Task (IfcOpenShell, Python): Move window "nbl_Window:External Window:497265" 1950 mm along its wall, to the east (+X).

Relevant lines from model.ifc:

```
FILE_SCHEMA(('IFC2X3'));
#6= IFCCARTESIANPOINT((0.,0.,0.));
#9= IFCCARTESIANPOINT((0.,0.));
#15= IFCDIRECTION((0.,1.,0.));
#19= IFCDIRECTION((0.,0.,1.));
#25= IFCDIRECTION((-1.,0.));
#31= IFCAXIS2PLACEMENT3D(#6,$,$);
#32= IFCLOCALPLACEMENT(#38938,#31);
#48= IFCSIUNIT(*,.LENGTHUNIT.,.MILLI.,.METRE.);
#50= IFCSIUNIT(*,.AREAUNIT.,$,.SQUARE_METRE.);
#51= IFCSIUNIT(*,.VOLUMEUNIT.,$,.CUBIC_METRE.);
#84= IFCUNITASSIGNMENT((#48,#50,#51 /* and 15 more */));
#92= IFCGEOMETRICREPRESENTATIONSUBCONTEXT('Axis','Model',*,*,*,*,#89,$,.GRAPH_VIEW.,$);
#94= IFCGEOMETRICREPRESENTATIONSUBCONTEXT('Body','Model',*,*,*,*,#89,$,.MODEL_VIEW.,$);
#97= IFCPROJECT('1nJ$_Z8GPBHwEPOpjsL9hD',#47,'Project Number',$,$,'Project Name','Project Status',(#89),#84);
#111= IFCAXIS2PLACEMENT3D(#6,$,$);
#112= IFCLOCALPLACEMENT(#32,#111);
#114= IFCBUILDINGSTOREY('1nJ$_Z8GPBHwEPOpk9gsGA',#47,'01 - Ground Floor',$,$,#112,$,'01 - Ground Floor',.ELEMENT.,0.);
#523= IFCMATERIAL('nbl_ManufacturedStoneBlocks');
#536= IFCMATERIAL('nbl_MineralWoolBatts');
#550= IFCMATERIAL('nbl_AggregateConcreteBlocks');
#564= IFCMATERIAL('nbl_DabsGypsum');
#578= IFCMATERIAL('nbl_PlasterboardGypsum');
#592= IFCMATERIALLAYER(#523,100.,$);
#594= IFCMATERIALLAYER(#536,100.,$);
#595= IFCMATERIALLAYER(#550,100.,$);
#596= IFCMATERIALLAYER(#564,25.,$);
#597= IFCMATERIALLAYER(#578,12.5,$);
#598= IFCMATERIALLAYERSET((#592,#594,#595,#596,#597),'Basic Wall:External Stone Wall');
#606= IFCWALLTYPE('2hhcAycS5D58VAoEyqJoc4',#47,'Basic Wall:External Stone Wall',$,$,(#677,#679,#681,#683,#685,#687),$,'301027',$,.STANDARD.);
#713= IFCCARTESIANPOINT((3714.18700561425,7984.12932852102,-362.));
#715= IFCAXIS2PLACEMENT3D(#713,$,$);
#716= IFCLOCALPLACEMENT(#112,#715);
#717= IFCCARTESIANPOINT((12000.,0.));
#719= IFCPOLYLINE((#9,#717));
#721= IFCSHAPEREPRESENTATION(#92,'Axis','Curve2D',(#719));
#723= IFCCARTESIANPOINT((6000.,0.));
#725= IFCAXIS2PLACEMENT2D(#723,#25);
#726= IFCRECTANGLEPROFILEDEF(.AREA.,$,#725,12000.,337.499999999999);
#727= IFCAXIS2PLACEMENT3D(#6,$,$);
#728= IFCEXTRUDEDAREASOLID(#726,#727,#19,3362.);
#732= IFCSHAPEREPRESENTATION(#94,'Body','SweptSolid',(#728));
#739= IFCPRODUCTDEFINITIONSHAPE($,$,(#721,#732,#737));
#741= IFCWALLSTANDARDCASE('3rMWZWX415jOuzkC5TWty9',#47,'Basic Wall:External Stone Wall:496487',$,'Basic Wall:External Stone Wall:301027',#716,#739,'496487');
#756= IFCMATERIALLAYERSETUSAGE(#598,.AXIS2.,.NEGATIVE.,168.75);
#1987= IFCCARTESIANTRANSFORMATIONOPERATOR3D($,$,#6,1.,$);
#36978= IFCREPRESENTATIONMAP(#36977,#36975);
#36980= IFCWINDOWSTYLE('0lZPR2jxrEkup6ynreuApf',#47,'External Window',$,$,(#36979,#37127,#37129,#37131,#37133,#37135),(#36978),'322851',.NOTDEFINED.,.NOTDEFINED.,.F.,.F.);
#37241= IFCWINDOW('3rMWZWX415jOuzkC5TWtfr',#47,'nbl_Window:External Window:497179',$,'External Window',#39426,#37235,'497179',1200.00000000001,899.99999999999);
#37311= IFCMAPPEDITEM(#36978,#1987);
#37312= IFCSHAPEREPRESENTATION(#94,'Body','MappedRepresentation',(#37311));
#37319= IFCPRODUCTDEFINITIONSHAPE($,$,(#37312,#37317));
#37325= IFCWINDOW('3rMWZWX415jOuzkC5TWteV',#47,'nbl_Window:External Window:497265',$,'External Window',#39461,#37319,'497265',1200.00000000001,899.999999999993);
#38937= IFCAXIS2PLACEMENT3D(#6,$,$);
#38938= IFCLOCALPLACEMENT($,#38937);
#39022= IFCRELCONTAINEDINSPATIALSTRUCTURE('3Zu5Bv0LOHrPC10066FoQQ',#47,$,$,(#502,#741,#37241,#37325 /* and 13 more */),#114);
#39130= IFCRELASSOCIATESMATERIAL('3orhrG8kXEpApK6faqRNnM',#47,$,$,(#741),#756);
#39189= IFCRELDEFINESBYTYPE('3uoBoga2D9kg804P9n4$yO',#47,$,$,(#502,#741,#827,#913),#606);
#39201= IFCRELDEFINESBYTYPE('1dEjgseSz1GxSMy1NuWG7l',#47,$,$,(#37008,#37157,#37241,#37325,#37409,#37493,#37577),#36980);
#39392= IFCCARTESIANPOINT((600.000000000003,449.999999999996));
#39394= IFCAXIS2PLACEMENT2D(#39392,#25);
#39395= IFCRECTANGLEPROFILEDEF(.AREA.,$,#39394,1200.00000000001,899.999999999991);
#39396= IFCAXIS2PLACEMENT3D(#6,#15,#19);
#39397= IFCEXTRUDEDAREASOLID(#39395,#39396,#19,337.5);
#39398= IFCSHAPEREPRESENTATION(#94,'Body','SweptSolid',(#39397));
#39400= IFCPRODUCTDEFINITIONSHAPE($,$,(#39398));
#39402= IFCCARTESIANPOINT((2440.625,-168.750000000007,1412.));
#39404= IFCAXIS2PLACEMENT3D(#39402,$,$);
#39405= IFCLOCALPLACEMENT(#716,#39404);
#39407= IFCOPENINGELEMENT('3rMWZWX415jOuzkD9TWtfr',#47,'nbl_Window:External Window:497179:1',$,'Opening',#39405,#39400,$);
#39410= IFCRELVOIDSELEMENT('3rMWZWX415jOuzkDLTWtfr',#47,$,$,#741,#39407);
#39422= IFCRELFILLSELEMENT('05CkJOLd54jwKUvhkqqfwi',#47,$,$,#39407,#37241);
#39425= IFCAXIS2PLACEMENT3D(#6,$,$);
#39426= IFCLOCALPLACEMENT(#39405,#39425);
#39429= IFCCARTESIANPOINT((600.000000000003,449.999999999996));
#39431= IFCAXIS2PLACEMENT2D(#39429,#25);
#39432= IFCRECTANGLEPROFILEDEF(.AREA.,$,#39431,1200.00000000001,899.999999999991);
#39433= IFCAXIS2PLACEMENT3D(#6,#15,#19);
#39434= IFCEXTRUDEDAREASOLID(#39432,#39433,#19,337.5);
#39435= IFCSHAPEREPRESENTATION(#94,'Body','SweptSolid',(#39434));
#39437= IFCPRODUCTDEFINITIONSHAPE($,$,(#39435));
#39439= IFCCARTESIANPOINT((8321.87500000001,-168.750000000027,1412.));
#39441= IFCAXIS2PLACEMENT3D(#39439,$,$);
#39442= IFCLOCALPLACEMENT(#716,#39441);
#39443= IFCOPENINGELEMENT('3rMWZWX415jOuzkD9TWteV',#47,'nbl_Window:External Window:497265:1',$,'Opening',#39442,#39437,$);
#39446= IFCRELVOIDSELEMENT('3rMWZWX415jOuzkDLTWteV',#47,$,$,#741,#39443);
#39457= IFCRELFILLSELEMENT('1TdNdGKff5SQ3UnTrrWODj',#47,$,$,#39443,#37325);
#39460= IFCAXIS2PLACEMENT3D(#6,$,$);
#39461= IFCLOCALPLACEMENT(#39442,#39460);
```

```python
import ifcopenshell
import ifcopenshell.api.geometry
import ifcopenshell.util.placement
import ifcopenshell.util.unit

model = ifcopenshell.open("model.ifc")
unit_scale = ifcopenshell.util.unit.calculate_unit_scale(model)

window = model.by_id(37325)
opening = window.FillsVoids[0].RelatingOpeningElement
wall = opening.VoidsElements[0].RelatingBuildingElement

wall_matrix = ifcopenshell.util.placement.get_local_placement(wall.ObjectPlacement)
shift = wall_matrix[:3, 0] * 1.95 / unit_scale
before = ifcopenshell.util.placement.get_local_placement(window.ObjectPlacement)[:3, 3].copy()

# The window is placed relative to its opening, so it follows when the opening moves.
matrix = ifcopenshell.util.placement.get_local_placement(opening.ObjectPlacement)
matrix[:3, 3] += shift
ifcopenshell.api.geometry.edit_object_placement(
    model, product=opening, matrix=matrix, is_si=False, should_transform_children=True
)

after = ifcopenshell.util.placement.get_local_placement(window.ObjectPlacement)[:3, 3]
print("window moved by", (after - before).round(3) + 0.0)

model.write("model-out.ifc")
```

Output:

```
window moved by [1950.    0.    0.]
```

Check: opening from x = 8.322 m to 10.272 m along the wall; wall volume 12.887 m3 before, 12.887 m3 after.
